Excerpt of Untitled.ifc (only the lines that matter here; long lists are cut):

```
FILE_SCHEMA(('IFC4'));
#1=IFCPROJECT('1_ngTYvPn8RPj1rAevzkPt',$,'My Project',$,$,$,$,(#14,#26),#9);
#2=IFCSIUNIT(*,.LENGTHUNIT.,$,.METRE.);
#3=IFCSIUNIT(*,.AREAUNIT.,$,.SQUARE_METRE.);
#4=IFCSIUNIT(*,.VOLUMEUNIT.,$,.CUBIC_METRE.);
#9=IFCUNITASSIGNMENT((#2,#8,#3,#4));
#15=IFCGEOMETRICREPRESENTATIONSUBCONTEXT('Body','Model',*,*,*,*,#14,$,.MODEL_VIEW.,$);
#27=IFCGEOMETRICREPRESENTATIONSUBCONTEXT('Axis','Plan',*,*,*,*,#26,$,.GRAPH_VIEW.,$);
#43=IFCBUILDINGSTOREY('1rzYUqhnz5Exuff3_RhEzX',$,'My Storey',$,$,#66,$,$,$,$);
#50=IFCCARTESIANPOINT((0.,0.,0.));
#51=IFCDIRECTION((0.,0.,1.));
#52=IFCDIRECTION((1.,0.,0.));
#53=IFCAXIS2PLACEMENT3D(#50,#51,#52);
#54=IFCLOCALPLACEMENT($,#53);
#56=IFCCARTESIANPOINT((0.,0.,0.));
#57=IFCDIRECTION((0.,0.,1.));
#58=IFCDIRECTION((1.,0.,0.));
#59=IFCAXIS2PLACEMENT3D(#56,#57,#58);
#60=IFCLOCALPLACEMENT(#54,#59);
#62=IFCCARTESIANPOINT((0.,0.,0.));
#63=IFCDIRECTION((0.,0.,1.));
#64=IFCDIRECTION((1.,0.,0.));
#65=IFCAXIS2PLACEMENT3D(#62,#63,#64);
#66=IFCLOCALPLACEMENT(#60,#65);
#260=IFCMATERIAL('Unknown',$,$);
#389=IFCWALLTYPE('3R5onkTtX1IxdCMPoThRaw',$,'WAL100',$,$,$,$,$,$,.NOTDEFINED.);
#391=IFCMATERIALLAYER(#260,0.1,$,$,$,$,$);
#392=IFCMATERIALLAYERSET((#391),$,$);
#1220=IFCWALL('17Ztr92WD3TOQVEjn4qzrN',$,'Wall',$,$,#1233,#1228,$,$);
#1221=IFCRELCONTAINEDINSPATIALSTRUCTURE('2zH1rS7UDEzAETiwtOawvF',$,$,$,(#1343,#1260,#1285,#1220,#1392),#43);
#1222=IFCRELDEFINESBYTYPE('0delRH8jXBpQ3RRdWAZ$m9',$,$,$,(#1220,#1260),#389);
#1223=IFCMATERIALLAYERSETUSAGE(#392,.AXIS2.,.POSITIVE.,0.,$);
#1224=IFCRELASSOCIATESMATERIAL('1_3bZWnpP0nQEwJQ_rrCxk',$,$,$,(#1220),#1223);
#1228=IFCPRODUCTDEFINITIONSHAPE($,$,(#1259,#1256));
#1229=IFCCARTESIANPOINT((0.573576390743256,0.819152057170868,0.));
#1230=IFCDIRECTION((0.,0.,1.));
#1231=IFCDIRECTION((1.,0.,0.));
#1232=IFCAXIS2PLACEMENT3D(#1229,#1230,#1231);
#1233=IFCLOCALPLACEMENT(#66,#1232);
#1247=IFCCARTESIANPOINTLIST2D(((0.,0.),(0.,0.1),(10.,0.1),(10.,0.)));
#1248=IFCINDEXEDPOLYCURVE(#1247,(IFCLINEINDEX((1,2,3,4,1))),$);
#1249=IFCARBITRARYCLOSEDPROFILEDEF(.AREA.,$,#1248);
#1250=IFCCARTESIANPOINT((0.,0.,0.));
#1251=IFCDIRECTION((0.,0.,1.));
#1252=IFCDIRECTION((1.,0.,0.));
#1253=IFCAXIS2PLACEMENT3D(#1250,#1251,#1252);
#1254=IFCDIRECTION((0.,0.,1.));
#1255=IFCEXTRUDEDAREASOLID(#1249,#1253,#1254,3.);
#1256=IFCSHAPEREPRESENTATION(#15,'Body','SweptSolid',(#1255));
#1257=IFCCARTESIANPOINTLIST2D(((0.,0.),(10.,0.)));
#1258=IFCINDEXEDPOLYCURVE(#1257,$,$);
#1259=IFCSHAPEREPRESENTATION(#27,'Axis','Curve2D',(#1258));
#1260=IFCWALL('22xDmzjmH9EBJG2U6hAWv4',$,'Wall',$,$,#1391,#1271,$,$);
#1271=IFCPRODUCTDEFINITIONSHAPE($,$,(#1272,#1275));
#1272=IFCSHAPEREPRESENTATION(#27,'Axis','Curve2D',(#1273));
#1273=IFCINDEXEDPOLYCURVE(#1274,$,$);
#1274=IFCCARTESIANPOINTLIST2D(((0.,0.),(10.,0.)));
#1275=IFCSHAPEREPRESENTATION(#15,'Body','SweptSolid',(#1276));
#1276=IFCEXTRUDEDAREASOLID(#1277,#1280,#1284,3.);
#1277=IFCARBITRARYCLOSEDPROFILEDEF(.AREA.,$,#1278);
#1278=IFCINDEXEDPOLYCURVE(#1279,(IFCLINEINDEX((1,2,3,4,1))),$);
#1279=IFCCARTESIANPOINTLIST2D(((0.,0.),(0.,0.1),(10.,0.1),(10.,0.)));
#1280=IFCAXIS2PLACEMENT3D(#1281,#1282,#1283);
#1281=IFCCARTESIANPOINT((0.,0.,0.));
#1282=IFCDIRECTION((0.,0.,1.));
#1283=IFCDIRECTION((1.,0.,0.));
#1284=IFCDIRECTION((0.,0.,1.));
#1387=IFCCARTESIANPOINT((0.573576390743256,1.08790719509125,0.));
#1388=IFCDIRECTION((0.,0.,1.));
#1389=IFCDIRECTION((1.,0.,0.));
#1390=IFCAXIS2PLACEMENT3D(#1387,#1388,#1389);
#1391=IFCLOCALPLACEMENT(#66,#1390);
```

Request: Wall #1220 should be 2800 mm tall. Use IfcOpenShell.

```python
import ifcopenshell
import ifcopenshell.geom
import ifcopenshell.util.representation
import ifcopenshell.util.shape
import ifcopenshell.util.unit

model = ifcopenshell.open("Untitled.ifc")
unit_scale = ifcopenshell.util.unit.calculate_unit_scale(model)
settings = ifcopenshell.geom.settings()


def volume(element):
    """Net volume in cubic metres, openings subtracted."""
    shape = ifcopenshell.geom.create_shape(settings, element)
    return ifcopenshell.util.shape.get_volume(shape.geometry)


wall = model.by_id(1220)
before = volume(wall)

body = ifcopenshell.util.representation.get_representation(wall, "Model", "Body")
solid = body.Items[0]
old_height = solid.Depth
solid.Depth = 2.8 / unit_scale
after = volume(wall)

print(f"height {old_height:g} -> {solid.Depth:g}, volume {before:.3f} -> {after:.3f} m3")

model.write("Untitled_rev.ifc")
```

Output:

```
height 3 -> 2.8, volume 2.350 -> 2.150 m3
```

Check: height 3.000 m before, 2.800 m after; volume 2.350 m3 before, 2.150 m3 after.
